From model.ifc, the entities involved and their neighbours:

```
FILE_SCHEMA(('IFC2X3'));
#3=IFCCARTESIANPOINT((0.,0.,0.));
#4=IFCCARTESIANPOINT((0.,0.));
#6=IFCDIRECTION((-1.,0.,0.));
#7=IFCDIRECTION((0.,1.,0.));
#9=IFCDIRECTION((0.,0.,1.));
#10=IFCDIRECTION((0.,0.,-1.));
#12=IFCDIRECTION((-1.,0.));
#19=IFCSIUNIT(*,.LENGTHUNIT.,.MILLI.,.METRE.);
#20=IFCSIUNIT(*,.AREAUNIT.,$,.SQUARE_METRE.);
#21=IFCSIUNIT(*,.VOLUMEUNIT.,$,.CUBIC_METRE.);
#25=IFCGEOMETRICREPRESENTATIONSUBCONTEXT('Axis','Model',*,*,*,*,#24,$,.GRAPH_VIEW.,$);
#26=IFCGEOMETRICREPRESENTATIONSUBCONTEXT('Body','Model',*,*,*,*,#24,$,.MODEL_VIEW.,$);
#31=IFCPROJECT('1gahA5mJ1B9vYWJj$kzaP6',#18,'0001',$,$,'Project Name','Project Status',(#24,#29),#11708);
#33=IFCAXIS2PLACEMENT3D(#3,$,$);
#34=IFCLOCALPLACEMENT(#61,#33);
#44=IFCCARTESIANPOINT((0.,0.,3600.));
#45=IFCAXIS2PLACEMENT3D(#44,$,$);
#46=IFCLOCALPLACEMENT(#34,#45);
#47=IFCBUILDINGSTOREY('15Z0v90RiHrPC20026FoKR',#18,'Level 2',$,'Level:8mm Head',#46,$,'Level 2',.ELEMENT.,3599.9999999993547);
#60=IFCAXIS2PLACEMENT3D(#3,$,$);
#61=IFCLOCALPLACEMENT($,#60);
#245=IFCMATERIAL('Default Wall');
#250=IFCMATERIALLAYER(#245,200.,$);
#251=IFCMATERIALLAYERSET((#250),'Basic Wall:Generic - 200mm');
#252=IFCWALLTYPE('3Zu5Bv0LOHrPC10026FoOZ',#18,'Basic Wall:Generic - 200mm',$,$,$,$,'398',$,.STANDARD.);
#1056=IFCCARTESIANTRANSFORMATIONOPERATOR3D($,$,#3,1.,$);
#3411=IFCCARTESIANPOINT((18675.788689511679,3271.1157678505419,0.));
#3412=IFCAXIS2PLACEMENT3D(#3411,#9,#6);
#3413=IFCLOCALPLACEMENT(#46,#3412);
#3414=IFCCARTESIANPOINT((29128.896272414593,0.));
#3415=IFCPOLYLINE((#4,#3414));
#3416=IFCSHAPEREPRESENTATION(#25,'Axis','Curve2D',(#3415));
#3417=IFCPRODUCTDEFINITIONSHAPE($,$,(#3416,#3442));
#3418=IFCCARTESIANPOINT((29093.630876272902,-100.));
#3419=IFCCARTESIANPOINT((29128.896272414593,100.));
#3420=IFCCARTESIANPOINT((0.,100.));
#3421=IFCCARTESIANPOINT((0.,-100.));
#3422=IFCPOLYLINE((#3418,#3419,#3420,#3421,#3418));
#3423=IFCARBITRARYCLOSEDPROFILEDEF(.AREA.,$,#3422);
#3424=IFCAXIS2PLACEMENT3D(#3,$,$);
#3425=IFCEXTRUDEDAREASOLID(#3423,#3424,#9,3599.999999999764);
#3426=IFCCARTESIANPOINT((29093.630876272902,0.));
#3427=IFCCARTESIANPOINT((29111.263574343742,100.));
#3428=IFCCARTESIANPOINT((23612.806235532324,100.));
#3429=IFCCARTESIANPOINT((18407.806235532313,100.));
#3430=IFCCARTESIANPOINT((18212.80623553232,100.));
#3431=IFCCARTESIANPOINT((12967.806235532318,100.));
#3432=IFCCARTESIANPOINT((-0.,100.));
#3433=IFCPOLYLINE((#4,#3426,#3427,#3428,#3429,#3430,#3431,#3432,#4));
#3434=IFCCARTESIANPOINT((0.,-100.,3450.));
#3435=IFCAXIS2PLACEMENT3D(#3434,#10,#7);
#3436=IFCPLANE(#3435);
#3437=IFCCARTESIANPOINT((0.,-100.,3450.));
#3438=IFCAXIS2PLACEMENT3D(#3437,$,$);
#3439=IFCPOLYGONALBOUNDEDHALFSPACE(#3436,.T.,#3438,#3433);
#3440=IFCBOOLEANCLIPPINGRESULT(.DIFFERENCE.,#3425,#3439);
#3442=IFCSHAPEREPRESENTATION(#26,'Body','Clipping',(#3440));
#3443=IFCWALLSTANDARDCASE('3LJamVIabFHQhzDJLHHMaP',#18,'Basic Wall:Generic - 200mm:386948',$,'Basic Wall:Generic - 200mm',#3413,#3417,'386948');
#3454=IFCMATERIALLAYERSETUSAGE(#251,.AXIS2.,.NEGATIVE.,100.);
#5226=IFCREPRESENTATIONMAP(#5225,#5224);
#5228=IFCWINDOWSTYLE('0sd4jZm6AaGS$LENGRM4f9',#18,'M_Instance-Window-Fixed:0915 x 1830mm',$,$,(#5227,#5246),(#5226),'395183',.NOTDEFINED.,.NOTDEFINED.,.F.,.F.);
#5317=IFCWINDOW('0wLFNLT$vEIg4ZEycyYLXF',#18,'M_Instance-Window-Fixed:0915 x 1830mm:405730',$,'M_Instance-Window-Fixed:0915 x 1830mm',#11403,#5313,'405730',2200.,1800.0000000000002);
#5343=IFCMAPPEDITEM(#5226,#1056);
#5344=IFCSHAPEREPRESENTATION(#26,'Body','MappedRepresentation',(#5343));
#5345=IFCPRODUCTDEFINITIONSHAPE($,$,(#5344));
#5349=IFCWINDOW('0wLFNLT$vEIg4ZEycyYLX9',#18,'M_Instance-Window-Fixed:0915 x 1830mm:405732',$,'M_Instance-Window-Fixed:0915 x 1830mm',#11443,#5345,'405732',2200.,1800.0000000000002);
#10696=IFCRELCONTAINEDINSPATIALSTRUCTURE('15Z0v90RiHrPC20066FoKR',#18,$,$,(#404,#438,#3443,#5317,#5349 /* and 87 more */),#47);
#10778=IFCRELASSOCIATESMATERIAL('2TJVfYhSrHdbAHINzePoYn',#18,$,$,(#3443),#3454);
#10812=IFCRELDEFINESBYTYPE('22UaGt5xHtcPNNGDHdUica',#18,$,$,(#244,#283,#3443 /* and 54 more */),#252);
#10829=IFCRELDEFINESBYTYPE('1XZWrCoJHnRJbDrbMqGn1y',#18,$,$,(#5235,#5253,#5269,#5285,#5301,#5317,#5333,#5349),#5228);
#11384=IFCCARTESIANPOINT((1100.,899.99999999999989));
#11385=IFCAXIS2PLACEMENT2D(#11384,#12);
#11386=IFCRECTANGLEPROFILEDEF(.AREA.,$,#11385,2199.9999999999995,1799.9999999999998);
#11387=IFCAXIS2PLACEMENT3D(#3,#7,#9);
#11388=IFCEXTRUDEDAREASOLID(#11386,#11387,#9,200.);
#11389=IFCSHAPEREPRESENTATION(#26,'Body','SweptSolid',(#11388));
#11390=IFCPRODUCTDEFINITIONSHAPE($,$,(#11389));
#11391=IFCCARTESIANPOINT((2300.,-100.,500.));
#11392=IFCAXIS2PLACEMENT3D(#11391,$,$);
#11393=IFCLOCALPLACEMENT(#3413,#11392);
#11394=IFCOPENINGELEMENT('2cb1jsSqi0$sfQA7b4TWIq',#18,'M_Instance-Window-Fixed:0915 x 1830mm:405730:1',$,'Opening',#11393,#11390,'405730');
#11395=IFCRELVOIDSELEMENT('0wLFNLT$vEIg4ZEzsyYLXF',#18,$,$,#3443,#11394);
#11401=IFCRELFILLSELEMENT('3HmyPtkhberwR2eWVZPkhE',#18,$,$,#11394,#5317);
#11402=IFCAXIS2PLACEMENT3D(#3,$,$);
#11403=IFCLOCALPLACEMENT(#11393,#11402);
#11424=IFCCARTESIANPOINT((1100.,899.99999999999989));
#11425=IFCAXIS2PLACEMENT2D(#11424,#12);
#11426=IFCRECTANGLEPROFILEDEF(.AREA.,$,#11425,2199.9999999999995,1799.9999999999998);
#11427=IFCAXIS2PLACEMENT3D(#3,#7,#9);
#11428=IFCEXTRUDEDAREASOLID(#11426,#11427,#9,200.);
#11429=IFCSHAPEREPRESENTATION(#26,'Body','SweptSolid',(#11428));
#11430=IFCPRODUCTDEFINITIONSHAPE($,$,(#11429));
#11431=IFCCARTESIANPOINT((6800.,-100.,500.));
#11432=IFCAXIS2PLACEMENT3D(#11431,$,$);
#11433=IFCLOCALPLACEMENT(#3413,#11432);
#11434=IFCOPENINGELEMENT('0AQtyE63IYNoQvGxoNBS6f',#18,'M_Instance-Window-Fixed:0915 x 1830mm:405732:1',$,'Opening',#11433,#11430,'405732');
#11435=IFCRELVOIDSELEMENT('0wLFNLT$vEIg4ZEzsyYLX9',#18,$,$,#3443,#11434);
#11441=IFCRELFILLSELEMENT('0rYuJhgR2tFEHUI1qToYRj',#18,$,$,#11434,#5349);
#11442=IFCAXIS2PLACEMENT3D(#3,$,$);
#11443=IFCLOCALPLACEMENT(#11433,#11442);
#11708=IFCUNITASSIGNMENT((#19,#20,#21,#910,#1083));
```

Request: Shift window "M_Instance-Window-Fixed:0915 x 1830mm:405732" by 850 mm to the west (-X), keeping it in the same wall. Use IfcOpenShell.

```python
import ifcopenshell
import ifcopenshell.api.geometry
import ifcopenshell.util.placement
import ifcopenshell.util.unit

model = ifcopenshell.open("model.ifc")
unit_scale = ifcopenshell.util.unit.calculate_unit_scale(model)

window = model.by_guid("0wLFNLT$vEIg4ZEycyYLX9")
opening = window.FillsVoids[0].RelatingOpeningElement
wall = opening.VoidsElements[0].RelatingBuildingElement

wall_matrix = ifcopenshell.util.placement.get_local_placement(wall.ObjectPlacement)
shift = wall_matrix[:3, 0] * 0.85 / unit_scale
before = ifcopenshell.util.placement.get_local_placement(window.ObjectPlacement)[:3, 3].copy()

# The window is placed relative to its opening, so it follows when the opening moves.
matrix = ifcopenshell.util.placement.get_local_placement(opening.ObjectPlacement)
matrix[:3, 3] += shift
ifcopenshell.api.geometry.edit_object_placement(
    model, product=opening, matrix=matrix, is_si=False, should_transform_children=True
)

after = ifcopenshell.util.placement.get_local_placement(window.ObjectPlacement)[:3, 3]
print("window moved by", (after - before).round(3) + 0.0)

model.write("model_v2.ifc")
```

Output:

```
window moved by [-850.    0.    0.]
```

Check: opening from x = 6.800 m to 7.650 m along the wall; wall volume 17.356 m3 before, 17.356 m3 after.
